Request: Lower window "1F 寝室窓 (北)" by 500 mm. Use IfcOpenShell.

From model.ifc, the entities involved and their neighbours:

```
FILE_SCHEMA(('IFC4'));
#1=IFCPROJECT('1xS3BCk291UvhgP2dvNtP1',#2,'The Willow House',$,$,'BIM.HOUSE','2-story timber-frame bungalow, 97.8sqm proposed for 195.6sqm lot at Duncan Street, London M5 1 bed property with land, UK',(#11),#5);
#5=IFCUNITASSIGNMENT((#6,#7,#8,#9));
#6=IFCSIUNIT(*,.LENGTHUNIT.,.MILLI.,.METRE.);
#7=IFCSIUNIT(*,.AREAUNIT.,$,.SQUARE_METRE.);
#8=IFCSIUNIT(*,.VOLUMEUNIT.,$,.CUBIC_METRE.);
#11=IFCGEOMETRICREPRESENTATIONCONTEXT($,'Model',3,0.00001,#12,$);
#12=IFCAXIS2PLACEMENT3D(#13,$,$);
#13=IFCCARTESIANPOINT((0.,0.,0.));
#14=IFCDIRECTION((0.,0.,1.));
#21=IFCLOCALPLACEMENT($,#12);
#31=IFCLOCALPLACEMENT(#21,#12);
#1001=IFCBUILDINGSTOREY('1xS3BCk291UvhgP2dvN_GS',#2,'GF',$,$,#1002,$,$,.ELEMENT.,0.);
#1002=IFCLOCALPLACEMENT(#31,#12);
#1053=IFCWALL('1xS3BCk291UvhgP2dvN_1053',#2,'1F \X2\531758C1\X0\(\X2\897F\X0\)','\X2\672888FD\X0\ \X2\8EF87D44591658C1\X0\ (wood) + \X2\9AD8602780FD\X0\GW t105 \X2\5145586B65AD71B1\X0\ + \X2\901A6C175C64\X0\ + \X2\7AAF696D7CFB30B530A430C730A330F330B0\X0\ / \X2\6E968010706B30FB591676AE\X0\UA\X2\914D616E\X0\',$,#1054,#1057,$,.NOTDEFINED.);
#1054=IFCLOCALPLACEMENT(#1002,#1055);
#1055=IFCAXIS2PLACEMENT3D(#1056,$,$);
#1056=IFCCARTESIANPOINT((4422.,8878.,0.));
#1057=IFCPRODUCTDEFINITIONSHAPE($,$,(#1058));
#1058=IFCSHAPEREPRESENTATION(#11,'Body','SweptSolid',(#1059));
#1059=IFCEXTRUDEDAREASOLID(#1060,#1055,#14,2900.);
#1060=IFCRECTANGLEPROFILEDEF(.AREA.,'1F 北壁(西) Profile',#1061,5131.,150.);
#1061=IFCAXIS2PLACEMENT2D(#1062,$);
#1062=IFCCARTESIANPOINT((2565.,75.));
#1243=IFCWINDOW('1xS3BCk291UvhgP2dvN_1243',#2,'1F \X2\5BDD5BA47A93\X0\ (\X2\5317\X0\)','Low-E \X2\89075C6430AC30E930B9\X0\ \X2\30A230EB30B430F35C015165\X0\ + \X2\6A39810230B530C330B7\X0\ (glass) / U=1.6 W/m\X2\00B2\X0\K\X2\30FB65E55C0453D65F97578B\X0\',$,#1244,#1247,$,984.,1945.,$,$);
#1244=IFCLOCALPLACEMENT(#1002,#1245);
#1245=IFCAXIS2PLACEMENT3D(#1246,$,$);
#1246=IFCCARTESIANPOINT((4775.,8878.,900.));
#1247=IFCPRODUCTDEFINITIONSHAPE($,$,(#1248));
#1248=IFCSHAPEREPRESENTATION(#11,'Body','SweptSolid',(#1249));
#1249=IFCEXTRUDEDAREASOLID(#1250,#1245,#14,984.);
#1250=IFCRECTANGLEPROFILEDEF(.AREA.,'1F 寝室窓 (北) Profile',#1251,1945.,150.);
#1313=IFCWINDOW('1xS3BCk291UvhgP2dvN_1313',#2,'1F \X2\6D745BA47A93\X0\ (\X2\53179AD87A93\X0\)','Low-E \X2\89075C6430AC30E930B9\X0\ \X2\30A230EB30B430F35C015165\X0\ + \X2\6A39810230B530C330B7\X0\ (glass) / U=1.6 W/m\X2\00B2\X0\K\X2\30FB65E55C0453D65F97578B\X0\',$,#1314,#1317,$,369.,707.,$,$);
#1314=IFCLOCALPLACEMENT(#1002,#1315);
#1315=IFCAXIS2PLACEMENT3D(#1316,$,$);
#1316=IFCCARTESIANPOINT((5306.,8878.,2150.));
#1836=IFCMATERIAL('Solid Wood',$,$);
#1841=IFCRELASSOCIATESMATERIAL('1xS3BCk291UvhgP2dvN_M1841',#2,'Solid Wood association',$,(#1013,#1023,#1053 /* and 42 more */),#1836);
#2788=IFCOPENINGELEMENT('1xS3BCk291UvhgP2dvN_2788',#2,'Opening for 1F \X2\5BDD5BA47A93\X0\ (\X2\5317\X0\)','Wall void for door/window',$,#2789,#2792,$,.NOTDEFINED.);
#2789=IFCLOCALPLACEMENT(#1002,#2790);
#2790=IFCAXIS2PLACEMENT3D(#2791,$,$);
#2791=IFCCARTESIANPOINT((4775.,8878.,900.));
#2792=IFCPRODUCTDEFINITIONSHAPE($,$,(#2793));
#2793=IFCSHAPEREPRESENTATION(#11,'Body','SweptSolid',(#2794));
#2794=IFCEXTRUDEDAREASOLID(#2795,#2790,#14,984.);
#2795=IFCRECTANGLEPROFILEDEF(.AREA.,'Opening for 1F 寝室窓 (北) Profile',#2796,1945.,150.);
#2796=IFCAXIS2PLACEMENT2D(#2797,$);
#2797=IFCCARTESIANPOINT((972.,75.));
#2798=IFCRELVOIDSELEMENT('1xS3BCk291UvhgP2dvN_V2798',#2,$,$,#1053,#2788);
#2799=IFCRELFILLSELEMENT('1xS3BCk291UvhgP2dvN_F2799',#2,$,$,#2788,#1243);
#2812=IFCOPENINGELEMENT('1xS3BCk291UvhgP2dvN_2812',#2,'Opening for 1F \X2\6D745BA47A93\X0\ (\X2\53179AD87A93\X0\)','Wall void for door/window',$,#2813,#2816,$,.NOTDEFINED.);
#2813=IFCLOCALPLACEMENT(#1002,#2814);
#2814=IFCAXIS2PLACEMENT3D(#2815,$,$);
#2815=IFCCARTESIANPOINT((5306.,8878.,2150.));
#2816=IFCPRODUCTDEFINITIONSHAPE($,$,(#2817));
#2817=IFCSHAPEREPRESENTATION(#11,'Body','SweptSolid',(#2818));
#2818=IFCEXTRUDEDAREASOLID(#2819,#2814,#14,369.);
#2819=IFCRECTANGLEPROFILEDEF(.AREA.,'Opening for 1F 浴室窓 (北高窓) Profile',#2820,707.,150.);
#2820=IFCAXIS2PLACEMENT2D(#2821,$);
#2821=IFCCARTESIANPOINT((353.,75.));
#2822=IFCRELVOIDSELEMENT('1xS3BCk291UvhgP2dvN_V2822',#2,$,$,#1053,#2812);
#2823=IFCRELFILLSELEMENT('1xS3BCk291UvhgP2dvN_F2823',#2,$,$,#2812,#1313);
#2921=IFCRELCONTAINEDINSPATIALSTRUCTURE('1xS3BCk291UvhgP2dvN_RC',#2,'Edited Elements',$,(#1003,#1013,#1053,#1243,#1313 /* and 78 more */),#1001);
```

```python
import numpy as np
import ifcopenshell
import ifcopenshell.api.geometry
import ifcopenshell.util.placement
import ifcopenshell.util.unit

model = ifcopenshell.open("model.ifc")
unit_scale = ifcopenshell.util.unit.calculate_unit_scale(model)

window = model.by_guid("1xS3BCk291UvhgP2dvN_1243")
opening = window.FillsVoids[0].RelatingOpeningElement
dz = -0.5 / unit_scale

shift = np.array([0.0, 0.0, dz])
# The window is not placed relative to its opening, so move both.
for product in (opening, window):
    matrix = ifcopenshell.util.placement.get_local_placement(product.ObjectPlacement)
    matrix[:3, 3] += shift
    ifcopenshell.api.geometry.edit_object_placement(model, product=product, matrix=matrix, is_si=False)

print(f"moved by {dz * unit_scale:+.3f} m")

model.write("model-out.ifc")
```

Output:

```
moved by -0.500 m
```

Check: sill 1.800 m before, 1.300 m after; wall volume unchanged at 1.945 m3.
